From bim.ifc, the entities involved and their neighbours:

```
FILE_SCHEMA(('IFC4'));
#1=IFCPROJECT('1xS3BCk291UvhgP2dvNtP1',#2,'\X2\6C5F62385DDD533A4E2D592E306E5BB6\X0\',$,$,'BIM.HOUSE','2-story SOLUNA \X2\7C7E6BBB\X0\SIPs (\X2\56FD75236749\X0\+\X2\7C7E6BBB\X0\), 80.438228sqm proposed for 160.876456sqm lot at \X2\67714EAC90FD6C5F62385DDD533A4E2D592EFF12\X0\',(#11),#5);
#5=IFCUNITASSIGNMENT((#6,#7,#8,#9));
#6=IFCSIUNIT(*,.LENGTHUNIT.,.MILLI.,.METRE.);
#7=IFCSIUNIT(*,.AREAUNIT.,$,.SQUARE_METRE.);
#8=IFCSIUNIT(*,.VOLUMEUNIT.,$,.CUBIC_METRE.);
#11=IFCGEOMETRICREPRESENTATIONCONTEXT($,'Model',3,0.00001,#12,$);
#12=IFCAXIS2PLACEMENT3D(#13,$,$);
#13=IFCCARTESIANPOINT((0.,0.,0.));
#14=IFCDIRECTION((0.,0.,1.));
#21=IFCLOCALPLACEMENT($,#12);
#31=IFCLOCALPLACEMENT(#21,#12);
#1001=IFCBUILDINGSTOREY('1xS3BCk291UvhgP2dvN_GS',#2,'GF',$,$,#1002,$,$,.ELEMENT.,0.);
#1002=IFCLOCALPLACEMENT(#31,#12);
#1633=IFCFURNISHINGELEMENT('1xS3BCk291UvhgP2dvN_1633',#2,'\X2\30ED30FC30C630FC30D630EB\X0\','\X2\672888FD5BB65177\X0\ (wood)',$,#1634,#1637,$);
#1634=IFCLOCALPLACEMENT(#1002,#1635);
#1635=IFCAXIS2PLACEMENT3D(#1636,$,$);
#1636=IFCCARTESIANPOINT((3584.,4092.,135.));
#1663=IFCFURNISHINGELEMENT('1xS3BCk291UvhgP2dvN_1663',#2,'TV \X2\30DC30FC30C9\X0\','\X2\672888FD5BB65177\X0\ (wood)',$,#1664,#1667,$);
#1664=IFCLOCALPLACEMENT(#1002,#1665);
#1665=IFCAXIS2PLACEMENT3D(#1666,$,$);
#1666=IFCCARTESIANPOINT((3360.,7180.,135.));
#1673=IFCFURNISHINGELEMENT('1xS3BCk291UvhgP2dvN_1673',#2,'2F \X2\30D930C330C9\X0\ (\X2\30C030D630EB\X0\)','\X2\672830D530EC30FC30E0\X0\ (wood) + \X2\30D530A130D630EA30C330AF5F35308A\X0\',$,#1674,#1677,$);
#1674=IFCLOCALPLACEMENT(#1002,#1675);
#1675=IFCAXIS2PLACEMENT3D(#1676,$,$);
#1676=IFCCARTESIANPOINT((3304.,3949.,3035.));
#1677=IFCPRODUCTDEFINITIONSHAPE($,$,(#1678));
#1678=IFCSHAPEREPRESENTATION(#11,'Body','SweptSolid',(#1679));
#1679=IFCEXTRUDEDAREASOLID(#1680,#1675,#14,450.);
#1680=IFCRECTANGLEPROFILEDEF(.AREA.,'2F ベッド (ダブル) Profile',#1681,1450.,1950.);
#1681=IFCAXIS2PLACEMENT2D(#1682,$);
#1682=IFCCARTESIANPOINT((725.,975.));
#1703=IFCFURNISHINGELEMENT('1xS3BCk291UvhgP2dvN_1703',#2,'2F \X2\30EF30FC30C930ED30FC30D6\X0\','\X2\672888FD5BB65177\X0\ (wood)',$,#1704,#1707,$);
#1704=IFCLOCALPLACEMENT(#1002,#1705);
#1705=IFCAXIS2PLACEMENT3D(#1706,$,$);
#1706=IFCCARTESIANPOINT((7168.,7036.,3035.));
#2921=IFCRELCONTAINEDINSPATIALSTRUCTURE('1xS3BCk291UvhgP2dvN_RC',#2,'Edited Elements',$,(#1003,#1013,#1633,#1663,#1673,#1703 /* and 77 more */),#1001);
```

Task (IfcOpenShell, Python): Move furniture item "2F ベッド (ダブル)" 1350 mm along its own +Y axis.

```python
import ifcopenshell
import ifcopenshell.api.geometry
import ifcopenshell.util.placement
import ifcopenshell.util.unit

model = ifcopenshell.open("bim.ifc")
unit_scale = ifcopenshell.util.unit.calculate_unit_scale(model)

item = model.by_guid("1xS3BCk291UvhgP2dvN_1673")
matrix = ifcopenshell.util.placement.get_local_placement(item.ObjectPlacement)
matrix[:3, 3] += matrix[:3, 1] * 1.35 / unit_scale
ifcopenshell.api.geometry.edit_object_placement(model, product=item, matrix=matrix, is_si=False)

print(ifcopenshell.util.placement.get_local_placement(item.ObjectPlacement).round(3) + 0.0)

model.write("bim_v2.ifc")
```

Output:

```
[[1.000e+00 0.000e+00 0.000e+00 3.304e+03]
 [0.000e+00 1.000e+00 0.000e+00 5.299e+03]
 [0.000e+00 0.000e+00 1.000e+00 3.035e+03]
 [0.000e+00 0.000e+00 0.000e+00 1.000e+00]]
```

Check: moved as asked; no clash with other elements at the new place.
